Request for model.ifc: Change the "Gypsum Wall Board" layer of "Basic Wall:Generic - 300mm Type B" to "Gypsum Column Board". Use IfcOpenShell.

First a look at what the model holds.

```python
import ifcopenshell
import ifcopenshell.util.element

model = ifcopenshell.open("model.ifc")
print(model.schema)
for layer_set in model.by_type("IfcMaterialLayerSet"):
    if layer_set.LayerSetName == "Basic Wall:Generic - 300mm Type B":
        for layer in layer_set.MaterialLayers:
            print(layer.id(), layer.Material and layer.Material.Name, layer.LayerThickness, sep=" | ")
        print(len(ifcopenshell.util.element.get_elements_by_material(model, layer_set)), "elements and types use it")
print(sorted(m.Name for m in model.by_type("IfcMaterial") if m.Name)[:60])
```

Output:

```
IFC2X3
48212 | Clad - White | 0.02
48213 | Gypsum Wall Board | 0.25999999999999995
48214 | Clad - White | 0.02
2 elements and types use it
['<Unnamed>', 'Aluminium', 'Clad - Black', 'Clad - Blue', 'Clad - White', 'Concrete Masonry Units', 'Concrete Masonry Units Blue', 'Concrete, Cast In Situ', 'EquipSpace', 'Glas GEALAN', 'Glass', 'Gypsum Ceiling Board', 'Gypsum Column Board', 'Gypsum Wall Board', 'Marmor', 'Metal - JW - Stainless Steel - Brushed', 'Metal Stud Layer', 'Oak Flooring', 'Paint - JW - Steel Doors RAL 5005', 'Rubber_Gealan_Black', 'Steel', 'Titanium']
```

```python
import ifcopenshell
import ifcopenshell.api.material

model = ifcopenshell.open("model.ifc")

layer_set = next(s for s in model.by_type("IfcMaterialLayerSet") if s.LayerSetName == "Basic Wall:Generic - 300mm Type B")
layer = next(l for l in layer_set.MaterialLayers if l.Material and l.Material.Name == "Gypsum Wall Board")
material = next(m for m in model.by_type("IfcMaterial") if m.Name == "Gypsum Column Board")

# Point this one layer at the other material; renaming the old one would change it everywhere.
ifcopenshell.api.material.edit_layer(model, layer=layer, attributes={}, material=material)

print([l.Material.Name if l.Material else None for l in layer_set.MaterialLayers])

model.write("model_edited.ifc")
```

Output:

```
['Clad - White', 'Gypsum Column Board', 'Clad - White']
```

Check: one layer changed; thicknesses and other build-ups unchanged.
